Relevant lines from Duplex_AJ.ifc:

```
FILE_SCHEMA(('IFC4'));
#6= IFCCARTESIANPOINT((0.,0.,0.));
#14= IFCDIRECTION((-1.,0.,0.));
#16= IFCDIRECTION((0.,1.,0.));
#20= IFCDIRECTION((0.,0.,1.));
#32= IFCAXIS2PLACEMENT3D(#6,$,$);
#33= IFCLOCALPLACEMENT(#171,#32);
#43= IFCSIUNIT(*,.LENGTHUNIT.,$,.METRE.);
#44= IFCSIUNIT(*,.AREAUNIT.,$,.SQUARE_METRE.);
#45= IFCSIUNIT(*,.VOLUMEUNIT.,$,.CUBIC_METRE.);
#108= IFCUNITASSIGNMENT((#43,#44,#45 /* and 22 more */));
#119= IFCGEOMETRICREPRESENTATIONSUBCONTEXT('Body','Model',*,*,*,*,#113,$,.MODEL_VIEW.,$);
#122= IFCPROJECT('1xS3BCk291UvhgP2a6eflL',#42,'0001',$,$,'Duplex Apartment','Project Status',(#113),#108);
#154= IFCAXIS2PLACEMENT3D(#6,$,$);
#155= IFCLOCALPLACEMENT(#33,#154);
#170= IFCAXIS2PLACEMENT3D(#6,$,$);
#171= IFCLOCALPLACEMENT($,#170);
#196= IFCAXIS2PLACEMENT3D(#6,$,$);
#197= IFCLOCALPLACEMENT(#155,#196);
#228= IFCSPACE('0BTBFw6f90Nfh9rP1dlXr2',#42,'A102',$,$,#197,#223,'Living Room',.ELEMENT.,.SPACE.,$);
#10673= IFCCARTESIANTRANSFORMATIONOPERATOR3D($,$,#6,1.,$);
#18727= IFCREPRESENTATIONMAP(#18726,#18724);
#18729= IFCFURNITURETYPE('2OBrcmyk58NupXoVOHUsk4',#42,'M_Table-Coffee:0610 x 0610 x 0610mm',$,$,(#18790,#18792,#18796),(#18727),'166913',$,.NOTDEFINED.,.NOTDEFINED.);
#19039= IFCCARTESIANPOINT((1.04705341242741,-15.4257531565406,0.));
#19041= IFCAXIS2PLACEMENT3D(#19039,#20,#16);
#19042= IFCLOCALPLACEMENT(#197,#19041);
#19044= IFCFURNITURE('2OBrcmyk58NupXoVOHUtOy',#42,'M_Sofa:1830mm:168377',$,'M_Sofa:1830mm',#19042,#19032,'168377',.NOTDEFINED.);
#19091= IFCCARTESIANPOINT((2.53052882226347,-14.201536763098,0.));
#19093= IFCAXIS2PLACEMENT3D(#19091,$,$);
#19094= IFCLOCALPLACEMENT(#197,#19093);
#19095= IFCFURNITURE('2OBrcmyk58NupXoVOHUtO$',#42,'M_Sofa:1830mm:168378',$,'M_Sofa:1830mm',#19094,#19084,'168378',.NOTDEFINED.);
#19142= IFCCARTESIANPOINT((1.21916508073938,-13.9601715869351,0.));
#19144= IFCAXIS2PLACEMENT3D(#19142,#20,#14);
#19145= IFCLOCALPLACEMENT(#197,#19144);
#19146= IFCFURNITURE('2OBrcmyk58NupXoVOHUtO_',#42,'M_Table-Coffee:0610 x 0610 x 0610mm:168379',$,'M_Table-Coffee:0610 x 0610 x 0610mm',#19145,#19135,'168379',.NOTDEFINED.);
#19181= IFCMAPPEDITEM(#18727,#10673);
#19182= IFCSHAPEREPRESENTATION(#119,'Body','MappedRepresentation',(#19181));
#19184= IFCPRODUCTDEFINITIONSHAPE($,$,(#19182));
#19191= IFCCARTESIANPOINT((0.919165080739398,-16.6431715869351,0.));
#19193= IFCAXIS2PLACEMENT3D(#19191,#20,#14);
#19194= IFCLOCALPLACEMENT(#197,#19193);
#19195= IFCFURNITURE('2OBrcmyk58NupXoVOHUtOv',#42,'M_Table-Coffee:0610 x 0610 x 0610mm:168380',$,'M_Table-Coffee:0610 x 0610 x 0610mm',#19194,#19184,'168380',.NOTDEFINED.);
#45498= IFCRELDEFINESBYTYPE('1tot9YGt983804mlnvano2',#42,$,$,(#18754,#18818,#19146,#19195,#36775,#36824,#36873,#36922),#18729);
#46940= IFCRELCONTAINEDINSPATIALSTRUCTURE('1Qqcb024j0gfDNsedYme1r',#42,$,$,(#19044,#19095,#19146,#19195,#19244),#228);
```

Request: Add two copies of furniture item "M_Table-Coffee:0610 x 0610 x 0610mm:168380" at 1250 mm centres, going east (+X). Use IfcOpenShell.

```python
import numpy as np
import ifcopenshell
import ifcopenshell.api.geometry
import ifcopenshell.api.root
import ifcopenshell.util.element
import ifcopenshell.util.placement
import ifcopenshell.util.unit

model = ifcopenshell.open("Duplex_AJ.ifc")
unit_scale = ifcopenshell.util.unit.calculate_unit_scale(model)


def reuse_history(source, copy):
    """copy_class also copies each property set's owner history, people and application; keep the originals."""
    for rel in copy.IsDefinedBy:
        if rel.is_a("IfcRelDefinesByProperties") and (history := rel.RelatingPropertyDefinition.OwnerHistory):
            rel.RelatingPropertyDefinition.OwnerHistory = source.OwnerHistory
            ifcopenshell.util.element.remove_deep2(model, history)


source = model.by_id(19195)
base = ifcopenshell.util.placement.get_local_placement(source.ObjectPlacement)
step = np.array([1.0, 0.0, 0.0]) * 1.25 / unit_scale

for i in range(1, 3):
    copy = ifcopenshell.api.root.copy_class(model, product=source)
    copy.Representation = ifcopenshell.util.element.copy_deep(
        model, source.Representation, exclude=["IfcGeometricRepresentationContext", "IfcRepresentationMap"]
    )
    copy.Name = "M_Table-Coffee:0610 x 0610 x 0610mm"
    copy.Tag = None
    reuse_history(source, copy)
    matrix = base.copy()
    matrix[:3, 3] += i * step
    print("added at", matrix[:3, 3].round(3) + 0.0)
    ifcopenshell.api.geometry.edit_object_placement(model, product=copy, matrix=matrix, is_si=False)

model.write("Duplex_AJ_v2.ifc")
```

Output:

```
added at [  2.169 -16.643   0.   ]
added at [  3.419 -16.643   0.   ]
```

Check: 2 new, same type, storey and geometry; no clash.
